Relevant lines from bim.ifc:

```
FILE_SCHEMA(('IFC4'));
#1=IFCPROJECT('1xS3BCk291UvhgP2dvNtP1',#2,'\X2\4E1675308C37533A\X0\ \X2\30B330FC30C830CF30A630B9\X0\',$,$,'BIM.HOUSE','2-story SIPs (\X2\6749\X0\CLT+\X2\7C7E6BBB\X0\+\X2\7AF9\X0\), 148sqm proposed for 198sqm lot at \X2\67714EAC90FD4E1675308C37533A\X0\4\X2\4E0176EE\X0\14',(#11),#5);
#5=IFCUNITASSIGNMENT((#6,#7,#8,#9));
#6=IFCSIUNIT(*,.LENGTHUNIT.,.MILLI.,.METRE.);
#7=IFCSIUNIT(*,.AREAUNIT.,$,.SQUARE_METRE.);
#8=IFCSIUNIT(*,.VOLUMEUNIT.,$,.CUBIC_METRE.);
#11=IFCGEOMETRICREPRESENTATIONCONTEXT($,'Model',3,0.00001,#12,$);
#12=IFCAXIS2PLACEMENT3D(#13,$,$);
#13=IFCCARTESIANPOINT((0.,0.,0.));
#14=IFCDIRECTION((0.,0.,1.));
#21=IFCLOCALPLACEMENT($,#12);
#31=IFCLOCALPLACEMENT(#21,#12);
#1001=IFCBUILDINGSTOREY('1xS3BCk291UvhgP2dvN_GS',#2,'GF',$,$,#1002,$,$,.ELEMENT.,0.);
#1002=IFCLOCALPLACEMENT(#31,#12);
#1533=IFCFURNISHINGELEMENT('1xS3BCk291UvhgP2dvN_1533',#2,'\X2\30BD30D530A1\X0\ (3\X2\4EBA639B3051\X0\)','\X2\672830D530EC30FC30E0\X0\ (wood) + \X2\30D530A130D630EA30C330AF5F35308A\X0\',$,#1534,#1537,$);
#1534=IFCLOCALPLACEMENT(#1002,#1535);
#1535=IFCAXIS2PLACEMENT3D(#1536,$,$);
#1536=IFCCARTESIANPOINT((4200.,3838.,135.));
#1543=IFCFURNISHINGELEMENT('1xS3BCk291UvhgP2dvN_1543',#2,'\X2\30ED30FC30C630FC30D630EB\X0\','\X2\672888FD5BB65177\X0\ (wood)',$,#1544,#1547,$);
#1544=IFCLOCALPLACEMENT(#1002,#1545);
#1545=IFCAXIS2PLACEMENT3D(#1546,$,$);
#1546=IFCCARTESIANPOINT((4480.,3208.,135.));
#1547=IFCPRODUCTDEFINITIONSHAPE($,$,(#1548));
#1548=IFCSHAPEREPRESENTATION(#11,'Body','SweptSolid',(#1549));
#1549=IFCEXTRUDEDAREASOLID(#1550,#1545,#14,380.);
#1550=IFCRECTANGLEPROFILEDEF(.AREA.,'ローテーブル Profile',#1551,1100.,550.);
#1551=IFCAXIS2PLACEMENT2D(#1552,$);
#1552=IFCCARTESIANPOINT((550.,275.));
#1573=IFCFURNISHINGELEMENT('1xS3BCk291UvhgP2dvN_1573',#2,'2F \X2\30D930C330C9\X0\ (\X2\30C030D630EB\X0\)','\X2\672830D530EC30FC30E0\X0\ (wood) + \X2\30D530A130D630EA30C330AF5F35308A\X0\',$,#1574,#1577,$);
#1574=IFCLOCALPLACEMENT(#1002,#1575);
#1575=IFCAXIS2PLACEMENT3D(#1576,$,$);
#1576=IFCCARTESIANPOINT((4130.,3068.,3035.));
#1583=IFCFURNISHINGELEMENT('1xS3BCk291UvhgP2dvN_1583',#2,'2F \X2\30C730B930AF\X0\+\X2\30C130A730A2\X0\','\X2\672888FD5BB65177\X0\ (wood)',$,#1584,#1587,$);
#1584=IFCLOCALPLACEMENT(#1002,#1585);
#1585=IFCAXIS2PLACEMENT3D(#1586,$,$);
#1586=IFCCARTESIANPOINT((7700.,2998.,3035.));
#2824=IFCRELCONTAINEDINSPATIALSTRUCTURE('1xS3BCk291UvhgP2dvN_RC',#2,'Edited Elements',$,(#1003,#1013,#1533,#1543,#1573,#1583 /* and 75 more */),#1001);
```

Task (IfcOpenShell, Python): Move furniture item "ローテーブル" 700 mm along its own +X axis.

```python
import ifcopenshell
import ifcopenshell.api.geometry
import ifcopenshell.util.placement
import ifcopenshell.util.unit

model = ifcopenshell.open("bim.ifc")
unit_scale = ifcopenshell.util.unit.calculate_unit_scale(model)

item = model.by_guid("1xS3BCk291UvhgP2dvN_1543")
matrix = ifcopenshell.util.placement.get_local_placement(item.ObjectPlacement)
matrix[:3, 3] += matrix[:3, 0] * 0.7 / unit_scale
ifcopenshell.api.geometry.edit_object_placement(model, product=item, matrix=matrix, is_si=False)

print(ifcopenshell.util.placement.get_local_placement(item.ObjectPlacement).round(3) + 0.0)

model.write("bim_updated.ifc")
```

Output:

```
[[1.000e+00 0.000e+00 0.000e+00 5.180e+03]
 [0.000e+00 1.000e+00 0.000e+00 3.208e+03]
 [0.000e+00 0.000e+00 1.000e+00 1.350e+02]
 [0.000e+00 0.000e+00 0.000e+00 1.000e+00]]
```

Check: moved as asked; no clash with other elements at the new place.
